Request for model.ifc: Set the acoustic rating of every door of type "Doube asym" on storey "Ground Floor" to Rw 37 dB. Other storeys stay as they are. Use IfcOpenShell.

First a look at what the model holds.

```python
import ifcopenshell
import ifcopenshell.util.element

model = ifcopenshell.open("model.ifc")
print(model.schema)
storey = next(s for s in model.by_type("IfcBuildingStorey") if s.Name == "Ground Floor")
doors = [e for e in ifcopenshell.util.element.get_decomposition(storey) if e.is_a("IfcDoor")]
seen = {}
for e in doors:
    element_type = ifcopenshell.util.element.get_type(e)
    key = (element_type.Name if element_type != e and element_type else None, ifcopenshell.util.element.get_pset(e, "Pset_DoorCommon", "AcousticRating"))
    seen[key] = seen.get(key, 0) + 1
for (name, value), count in sorted(seen.items(), key=str):
    print(count, "x", name, "|", value)
```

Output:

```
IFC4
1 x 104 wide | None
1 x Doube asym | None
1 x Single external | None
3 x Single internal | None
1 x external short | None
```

```python
import ifcopenshell
import ifcopenshell.api.pset
import ifcopenshell.util.element

model = ifcopenshell.open("model.ifc")

storey = next(s for s in model.by_type("IfcBuildingStorey") if s.Name == "Ground Floor")
doors = [e for e in ifcopenshell.util.element.get_decomposition(storey) if e.is_a("IfcDoor")]

count = 0
for e in doors:
    element_type = ifcopenshell.util.element.get_type(e)
    if element_type in (None, e) or element_type.Name != "Doube asym":
        continue
    # add_pset returns the element's existing set when there is one.
    pset = ifcopenshell.api.pset.add_pset(model, product=e, name="Pset_DoorCommon")
    ifcopenshell.api.pset.edit_pset(model, pset=pset, properties={"AcousticRating": "Rw 37 dB"})
    count += 1

print(count, "doors updated")

model.write("model-out.ifc")
```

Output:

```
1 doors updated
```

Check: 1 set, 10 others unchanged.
